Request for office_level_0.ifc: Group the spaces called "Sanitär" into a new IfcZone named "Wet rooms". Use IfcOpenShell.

First a look at what the model holds.

```python
import ifcopenshell

model = ifcopenshell.open("office_level_0.ifc")
print(model.schema)
seen = {}
for space in model.by_type("IfcSpace"):
    seen[space.LongName] = seen.get(space.LongName, 0) + 1
for name, count in sorted(seen.items(), key=str):
    print(count, "x", name)
print("zones:", [z.Name for z in model.by_type("IfcZone")][:20])
```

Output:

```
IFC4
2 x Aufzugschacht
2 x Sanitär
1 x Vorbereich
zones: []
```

```python
import ifcopenshell
import ifcopenshell.api.group
import ifcopenshell.api.root

model = ifcopenshell.open("office_level_0.ifc")

names = {"Sanitär"}
spaces = [s for s in model.by_type("IfcSpace") if s.LongName in names]

zone = ifcopenshell.api.root.create_entity(model, ifc_class="IfcZone", name="Wet rooms")
ifcopenshell.api.group.assign_group(model, products=spaces, group=zone)
print(len(spaces), "spaces in", zone.Name)

model.write("office_level_0_rev.ifc")
```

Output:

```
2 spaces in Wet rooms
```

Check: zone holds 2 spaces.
